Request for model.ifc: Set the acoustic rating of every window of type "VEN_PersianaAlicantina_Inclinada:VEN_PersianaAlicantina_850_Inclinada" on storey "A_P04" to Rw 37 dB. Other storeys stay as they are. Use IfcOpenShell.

First a look at what the model holds.

```python
import ifcopenshell
import ifcopenshell.util.element

model = ifcopenshell.open("model.ifc")
print(model.schema)
storey = next(s for s in model.by_type("IfcBuildingStorey") if s.Name == "A_P04")
windows = [e for e in ifcopenshell.util.element.get_decomposition(storey) if e.is_a("IfcWindow")]
seen = {}
for e in windows:
    element_type = ifcopenshell.util.element.get_type(e)
    key = (element_type.Name if element_type != e and element_type else None, ifcopenshell.util.element.get_pset(e, "Pset_WindowCommon", "AcousticRating"))
    seen[key] = seen.get(key, 0) + 1
for (name, value), count in sorted(seen.items(), key=str):
    print(count, "x", name, "|", value)
```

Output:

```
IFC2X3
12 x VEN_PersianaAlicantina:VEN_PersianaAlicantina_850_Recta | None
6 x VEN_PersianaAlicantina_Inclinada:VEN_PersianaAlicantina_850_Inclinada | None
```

```python
import ifcopenshell
import ifcopenshell.api.pset
import ifcopenshell.util.element

model = ifcopenshell.open("model.ifc")

storey = next(s for s in model.by_type("IfcBuildingStorey") if s.Name == "A_P04")
windows = [e for e in ifcopenshell.util.element.get_decomposition(storey) if e.is_a("IfcWindow")]

count = 0
for e in windows:
    element_type = ifcopenshell.util.element.get_type(e)
    if element_type in (None, e) or element_type.Name != "VEN_PersianaAlicantina_Inclinada:VEN_PersianaAlicantina_850_Inclinada":
        continue
    # add_pset returns the element's existing set when there is one.
    pset = ifcopenshell.api.pset.add_pset(model, product=e, name="Pset_WindowCommon")
    ifcopenshell.api.pset.edit_pset(model, pset=pset, properties={"AcousticRating": "Rw 37 dB"})
    count += 1

print(count, "windows updated")

model.write("model_updated.ifc")
```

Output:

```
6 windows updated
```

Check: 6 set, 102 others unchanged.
